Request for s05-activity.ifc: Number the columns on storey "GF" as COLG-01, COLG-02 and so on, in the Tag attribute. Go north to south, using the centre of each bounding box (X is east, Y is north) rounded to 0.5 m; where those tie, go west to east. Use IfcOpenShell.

First a look at what the model holds.

```python
import ifcopenshell
import ifcopenshell.util.element
import ifcopenshell.util.placement

model = ifcopenshell.open("s05-activity.ifc")
print(model.schema)
storey = next(s for s in model.by_type("IfcBuildingStorey") if s.Name == "GF")
columns = [e for e in ifcopenshell.util.element.get_decomposition(storey) if e.is_a("IfcColumn")]
for e in sorted(columns, key=lambda e: e.id()):
    origin = ifcopenshell.util.placement.get_local_placement(e.ObjectPlacement)[:3, 3]
    print(e.id(), e.Tag, e.Name, origin.round(2) + 0.0, sep=" | ")
```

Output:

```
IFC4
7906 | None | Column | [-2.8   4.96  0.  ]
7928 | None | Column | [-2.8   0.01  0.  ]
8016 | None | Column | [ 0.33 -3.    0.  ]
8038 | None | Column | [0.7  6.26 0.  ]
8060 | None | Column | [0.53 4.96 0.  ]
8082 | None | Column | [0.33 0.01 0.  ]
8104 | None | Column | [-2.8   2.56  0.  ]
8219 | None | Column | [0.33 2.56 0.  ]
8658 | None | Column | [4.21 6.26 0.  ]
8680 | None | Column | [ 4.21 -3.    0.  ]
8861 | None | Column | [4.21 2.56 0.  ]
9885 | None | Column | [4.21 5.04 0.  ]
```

```python
import ifcopenshell
import ifcopenshell.geom
import ifcopenshell.util.element
import ifcopenshell.util.shape

model = ifcopenshell.open("s05-activity.ifc")
settings = ifcopenshell.geom.settings()
settings.set("use-world-coords", True)


def centre(element):
    shape = ifcopenshell.geom.create_shape(settings, element)
    return ifcopenshell.util.shape.get_bbox_centroid(shape.geometry)


storey = next(s for s in model.by_type("IfcBuildingStorey") if s.Name == "GF")
columns = [e for e in ifcopenshell.util.element.get_decomposition(storey) if e.is_a("IfcColumn")]

# Insertion points can sit at a corner or the storey origin, so sort by the geometry (in metres).
centres = {e: centre(e) for e in columns}
columns.sort(key=lambda e: (-round(centres[e][1] / 0.5), centres[e][0]))

for i, e in enumerate(columns, start=1):
    number = f"COLG-{i:02d}"
    e.Tag = number
    print(e.id(), number)

model.write("s05-activity-out.ifc")
```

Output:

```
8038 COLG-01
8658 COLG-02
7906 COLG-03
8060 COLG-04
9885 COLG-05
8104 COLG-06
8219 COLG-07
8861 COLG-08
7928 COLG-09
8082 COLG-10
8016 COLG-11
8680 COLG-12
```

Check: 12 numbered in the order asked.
